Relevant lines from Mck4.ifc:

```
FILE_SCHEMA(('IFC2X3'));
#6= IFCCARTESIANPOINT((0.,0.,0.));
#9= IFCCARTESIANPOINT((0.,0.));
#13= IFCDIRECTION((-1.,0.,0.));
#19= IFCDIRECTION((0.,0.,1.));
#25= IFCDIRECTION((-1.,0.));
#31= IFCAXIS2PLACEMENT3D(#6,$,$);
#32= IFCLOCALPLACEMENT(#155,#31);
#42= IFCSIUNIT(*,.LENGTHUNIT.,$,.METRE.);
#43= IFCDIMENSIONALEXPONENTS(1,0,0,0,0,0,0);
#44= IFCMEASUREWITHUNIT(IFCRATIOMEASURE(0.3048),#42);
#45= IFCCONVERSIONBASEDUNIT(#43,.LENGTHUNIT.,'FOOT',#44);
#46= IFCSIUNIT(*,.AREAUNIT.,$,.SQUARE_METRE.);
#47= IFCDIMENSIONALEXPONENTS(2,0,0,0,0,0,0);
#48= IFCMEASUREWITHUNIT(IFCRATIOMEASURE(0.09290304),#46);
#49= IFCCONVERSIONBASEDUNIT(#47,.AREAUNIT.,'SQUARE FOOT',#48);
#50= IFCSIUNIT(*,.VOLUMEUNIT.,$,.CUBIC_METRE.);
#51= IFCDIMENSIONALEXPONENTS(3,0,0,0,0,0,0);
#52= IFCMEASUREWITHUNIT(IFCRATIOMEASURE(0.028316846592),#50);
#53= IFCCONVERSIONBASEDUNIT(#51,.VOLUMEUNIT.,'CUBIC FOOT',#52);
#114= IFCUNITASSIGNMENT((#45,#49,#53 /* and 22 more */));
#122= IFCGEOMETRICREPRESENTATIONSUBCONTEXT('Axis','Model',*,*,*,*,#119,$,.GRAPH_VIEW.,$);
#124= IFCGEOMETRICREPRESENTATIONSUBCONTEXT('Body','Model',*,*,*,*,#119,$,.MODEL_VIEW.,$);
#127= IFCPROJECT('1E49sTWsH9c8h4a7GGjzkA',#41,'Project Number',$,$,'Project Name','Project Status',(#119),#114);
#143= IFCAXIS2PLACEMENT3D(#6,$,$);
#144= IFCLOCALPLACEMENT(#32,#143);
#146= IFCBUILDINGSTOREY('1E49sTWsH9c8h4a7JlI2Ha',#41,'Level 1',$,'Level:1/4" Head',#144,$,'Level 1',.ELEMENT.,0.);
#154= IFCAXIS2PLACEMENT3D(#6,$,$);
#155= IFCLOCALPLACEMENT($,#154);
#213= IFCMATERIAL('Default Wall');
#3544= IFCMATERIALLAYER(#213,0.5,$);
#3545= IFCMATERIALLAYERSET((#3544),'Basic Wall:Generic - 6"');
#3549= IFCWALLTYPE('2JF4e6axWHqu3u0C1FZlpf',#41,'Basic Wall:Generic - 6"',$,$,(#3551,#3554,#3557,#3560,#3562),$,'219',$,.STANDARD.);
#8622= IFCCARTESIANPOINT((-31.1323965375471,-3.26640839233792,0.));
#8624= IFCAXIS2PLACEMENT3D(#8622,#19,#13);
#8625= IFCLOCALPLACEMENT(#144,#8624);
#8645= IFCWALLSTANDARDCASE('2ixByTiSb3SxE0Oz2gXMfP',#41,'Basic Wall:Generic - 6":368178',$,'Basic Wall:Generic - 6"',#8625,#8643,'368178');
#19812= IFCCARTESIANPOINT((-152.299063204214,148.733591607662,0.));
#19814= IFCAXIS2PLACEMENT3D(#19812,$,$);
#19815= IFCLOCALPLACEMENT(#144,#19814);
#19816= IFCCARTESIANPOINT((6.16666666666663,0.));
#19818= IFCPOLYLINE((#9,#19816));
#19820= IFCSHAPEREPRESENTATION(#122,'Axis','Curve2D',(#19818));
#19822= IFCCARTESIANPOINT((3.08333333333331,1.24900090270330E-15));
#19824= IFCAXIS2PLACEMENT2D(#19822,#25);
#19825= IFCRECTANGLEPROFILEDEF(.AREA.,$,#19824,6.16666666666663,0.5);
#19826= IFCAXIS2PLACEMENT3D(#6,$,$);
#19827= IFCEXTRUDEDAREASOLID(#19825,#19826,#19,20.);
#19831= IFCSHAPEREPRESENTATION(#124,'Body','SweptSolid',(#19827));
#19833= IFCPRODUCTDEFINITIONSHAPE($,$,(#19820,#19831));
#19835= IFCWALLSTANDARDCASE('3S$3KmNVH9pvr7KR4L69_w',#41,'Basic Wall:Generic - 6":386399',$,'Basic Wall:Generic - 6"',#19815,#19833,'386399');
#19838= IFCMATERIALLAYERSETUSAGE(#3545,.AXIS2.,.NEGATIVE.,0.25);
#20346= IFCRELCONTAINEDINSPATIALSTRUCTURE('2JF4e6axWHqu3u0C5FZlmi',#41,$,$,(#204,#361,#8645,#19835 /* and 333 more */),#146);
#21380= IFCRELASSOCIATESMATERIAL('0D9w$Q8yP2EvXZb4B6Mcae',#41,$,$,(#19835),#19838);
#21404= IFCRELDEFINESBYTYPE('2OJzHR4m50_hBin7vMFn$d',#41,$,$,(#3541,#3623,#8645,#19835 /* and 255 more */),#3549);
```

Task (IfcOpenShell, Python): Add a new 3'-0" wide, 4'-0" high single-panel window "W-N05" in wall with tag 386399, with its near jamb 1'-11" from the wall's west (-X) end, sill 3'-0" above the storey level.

```python
import numpy as np
import ifcopenshell
import ifcopenshell.api.feature
import ifcopenshell.api.geometry
import ifcopenshell.api.root
import ifcopenshell.api.spatial
import ifcopenshell.api.type
import ifcopenshell.geom
import ifcopenshell.util.element
import ifcopenshell.util.placement
import ifcopenshell.util.representation
import ifcopenshell.util.shape
import ifcopenshell.util.unit

model = ifcopenshell.open("Mck4.ifc")
unit_scale = ifcopenshell.util.unit.calculate_unit_scale(model)
settings = ifcopenshell.geom.settings()


def volume(element):
    """Net volume in cubic metres, openings subtracted."""
    shape = ifcopenshell.geom.create_shape(settings, element)
    return ifcopenshell.util.shape.get_volume(shape.geometry)


wall = model.by_guid("3S$3KmNVH9pvr7KR4L69_w")
storey = ifcopenshell.util.element.get_container(wall, ifc_class="IfcBuildingStorey")
context = ifcopenshell.util.representation.get_context(model, "Model", "Body", "MODEL_VIEW")
before = volume(wall)

width, height, from_end, sill = 0.9144, 1.2192, 0.5842, 0.9144  # metres

# The wall runs along its own X axis, and the end named is its -X end.
wall_shape = ifcopenshell.geom.create_shape(settings, wall)
x, y, z = ifcopenshell.util.shape.get_vertices(wall_shape.geometry).T
start = x.min() + from_end
face, thickness = float(y.min()), float(y.max() - y.min())
wall_matrix = ifcopenshell.util.placement.get_local_placement(wall.ObjectPlacement)
level = ifcopenshell.util.placement.get_local_placement(storey.ObjectPlacement)[2, 3]


def in_wall(x, y):
    """Placement at x, y metres in the wall's axes, at sill height."""
    matrix = wall_matrix.copy()
    matrix[:, 3] = wall_matrix @ np.array([x / unit_scale, y / unit_scale, 0.0, 1.0])
    matrix[2, 3] = level + sill / unit_scale
    return matrix


# Opening: a box that overshoots both wall faces by 50 mm.
opening = ifcopenshell.api.root.create_entity(model, ifc_class="IfcOpeningElement")
box = ifcopenshell.api.geometry.add_wall_representation(
    model, context=context, length=width, height=height, thickness=thickness + 0.1
)
ifcopenshell.api.geometry.assign_representation(model, product=opening, representation=box)
ifcopenshell.api.geometry.edit_object_placement(model, product=opening, matrix=in_wall(start, face - 0.05), is_si=False)
ifcopenshell.api.feature.add_feature(model, feature=opening, element=wall)

window = ifcopenshell.api.root.create_entity(model, ifc_class="IfcWindow", name="W-N05")
window.OverallWidth, window.OverallHeight = width / unit_scale, height / unit_scale
body = ifcopenshell.api.geometry.add_window_representation(
    model,
    context=context,
    overall_width=window.OverallWidth,
    overall_height=window.OverallHeight,
    partition_type="SINGLE_PANEL",
)
ifcopenshell.api.geometry.assign_representation(model, product=window, representation=body)
ifcopenshell.api.spatial.assign_container(model, products=[window], relating_structure=storey)
fills = ifcopenshell.api.feature.add_filling(model, opening=opening, element=window)
fills.OwnerHistory = window.OwnerHistory  # required in IFC2X3

# IFC2X3 keeps the operation on the window style.
style = ifcopenshell.api.root.create_entity(model, ifc_class="IfcWindowStyle", name="W-N05")
style.OperationType, style.ConstructionType = "SINGLE_PANEL", "NOTDEFINED"
style.ParameterTakesPrecedence = style.Sizeable = False
ifcopenshell.api.type.assign_type(model, related_objects=[window], relating_type=style)

# Centre the window in the wall's thickness.
ifcopenshell.api.geometry.edit_object_placement(model, product=window, matrix=in_wall(start, face), is_si=False)
window_shape = ifcopenshell.geom.create_shape(settings, window)
depth = ifcopenshell.util.shape.get_vertices(window_shape.geometry)[:, 1]
offset = face + thickness / 2 - (depth.min() + depth.max()) / 2
ifcopenshell.api.geometry.edit_object_placement(model, product=window, matrix=in_wall(start, offset), is_si=False)

after = volume(wall)

print(f"wall volume {before:.3f} -> {after:.3f} m3")

model.write("Mck4_edited.ifc")
```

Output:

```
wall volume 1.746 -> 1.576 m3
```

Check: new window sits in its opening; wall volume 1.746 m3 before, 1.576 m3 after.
